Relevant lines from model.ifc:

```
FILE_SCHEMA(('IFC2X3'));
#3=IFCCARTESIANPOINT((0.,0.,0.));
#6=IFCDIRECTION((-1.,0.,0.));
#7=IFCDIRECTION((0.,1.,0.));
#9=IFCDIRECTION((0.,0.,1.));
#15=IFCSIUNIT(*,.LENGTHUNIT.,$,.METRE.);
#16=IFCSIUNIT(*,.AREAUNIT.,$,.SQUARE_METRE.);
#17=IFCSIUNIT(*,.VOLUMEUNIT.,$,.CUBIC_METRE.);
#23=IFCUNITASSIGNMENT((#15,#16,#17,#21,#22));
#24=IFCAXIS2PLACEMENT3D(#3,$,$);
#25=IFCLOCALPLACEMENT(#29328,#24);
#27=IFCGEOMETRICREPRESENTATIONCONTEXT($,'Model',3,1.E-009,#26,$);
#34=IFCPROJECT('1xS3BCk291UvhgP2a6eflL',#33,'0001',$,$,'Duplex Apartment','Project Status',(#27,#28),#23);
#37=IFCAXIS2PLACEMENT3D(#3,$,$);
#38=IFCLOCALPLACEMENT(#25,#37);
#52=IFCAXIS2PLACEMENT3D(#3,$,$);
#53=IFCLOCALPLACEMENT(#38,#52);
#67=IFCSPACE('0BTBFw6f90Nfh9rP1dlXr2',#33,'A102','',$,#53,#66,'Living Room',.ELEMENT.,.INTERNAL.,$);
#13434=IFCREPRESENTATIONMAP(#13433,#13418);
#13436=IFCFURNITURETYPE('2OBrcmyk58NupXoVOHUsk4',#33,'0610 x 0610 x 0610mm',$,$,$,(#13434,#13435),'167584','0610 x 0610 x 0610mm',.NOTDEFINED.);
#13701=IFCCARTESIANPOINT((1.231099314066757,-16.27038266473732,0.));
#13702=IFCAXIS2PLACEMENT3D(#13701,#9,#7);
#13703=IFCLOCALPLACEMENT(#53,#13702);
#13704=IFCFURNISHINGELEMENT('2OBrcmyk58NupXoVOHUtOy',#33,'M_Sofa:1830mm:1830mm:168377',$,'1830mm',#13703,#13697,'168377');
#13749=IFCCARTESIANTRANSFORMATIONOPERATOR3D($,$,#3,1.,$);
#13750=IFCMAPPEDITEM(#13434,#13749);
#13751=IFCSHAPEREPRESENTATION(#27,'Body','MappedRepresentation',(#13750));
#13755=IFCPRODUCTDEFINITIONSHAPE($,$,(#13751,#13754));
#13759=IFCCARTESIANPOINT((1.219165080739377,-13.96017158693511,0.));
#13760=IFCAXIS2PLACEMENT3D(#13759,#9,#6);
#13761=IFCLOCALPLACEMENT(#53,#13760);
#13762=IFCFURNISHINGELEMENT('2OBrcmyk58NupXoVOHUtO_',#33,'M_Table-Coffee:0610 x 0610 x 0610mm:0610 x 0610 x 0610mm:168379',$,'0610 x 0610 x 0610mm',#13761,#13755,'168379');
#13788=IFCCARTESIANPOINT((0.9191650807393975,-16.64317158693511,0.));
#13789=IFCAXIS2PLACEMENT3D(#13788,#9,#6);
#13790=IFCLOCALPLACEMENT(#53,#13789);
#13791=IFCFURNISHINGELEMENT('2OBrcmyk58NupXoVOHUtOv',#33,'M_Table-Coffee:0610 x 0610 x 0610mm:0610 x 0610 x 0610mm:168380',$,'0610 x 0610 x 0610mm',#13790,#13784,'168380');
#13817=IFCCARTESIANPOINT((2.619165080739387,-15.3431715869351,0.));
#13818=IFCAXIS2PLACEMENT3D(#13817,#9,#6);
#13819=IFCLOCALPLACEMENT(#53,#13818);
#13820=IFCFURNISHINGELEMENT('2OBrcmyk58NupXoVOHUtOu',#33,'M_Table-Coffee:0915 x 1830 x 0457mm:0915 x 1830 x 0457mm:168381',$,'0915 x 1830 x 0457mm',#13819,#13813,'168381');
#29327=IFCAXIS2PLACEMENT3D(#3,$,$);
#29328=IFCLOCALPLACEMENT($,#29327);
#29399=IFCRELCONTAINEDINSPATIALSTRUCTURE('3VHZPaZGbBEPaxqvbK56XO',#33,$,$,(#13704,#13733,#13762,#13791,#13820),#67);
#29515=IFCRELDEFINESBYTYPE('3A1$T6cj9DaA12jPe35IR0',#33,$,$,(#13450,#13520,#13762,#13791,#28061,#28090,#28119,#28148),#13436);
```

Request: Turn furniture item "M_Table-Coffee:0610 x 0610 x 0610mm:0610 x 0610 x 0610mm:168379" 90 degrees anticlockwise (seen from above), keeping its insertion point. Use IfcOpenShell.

```python
import ifcopenshell
import ifcopenshell.api.geometry
import ifcopenshell.util.placement

model = ifcopenshell.open("model.ifc")

item = model.by_guid("2OBrcmyk58NupXoVOHUtO_")
matrix = ifcopenshell.util.placement.get_local_placement(item.ObjectPlacement)
matrix = matrix @ ifcopenshell.util.placement.rotation(90, "Z")
ifcopenshell.api.geometry.edit_object_placement(model, product=item, matrix=matrix, is_si=False)

print(ifcopenshell.util.placement.get_local_placement(item.ObjectPlacement).round(3) + 0.0)

model.write("model_v2.ifc")
```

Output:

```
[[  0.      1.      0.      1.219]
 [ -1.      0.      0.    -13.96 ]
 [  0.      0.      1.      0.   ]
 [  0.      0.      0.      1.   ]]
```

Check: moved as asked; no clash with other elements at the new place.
